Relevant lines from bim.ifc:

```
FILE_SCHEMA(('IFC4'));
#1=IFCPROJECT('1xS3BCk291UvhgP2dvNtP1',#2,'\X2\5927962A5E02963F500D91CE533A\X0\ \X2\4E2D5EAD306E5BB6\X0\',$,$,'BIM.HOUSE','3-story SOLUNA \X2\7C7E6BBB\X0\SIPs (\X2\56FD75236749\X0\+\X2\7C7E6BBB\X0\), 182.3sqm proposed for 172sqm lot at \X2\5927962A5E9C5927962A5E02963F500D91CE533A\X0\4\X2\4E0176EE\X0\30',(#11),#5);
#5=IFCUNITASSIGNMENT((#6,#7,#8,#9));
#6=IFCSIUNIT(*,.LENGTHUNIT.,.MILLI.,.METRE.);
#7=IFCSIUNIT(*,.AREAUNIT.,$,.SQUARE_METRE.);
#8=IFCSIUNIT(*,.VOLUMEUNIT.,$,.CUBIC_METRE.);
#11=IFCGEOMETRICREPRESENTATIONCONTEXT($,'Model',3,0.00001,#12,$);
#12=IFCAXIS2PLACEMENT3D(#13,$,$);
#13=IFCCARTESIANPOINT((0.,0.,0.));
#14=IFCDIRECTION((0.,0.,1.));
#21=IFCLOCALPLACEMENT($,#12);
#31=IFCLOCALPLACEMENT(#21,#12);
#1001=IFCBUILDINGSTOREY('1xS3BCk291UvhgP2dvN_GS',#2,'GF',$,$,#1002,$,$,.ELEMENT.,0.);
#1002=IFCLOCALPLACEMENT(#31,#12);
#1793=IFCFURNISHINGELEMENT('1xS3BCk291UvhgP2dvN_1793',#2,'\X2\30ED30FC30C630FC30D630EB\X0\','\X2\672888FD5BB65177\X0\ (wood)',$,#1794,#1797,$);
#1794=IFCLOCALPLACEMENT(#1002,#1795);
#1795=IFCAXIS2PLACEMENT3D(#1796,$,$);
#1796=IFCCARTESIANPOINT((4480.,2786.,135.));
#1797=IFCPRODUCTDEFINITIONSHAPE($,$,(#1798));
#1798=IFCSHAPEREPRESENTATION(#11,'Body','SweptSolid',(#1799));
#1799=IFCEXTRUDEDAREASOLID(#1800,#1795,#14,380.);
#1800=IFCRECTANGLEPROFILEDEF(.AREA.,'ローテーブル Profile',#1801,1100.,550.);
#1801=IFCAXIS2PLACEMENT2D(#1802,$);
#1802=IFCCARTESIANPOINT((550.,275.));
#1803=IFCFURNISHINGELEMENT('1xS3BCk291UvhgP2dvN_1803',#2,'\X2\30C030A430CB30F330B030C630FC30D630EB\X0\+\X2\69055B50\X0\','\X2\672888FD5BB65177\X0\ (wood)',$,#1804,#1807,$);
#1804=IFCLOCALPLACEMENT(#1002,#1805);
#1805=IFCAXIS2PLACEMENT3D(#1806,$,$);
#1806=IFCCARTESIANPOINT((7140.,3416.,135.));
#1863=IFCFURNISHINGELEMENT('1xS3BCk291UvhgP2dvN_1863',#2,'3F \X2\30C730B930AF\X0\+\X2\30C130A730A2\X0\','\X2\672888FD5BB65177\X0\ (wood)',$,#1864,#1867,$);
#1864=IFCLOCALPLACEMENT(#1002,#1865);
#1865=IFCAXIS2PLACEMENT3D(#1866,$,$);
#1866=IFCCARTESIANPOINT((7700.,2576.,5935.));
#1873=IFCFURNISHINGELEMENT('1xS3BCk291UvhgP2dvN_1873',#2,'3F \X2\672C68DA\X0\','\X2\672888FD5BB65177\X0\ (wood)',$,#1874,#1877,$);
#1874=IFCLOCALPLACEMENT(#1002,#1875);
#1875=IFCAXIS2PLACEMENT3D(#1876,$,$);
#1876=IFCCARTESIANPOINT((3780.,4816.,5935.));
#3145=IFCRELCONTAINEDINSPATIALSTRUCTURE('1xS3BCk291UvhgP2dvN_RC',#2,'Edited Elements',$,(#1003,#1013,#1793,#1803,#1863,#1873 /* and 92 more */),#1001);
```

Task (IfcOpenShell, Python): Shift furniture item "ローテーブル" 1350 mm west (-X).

```python
import ifcopenshell
import ifcopenshell.api.geometry
import ifcopenshell.util.placement
import ifcopenshell.util.unit

model = ifcopenshell.open("bim.ifc")
unit_scale = ifcopenshell.util.unit.calculate_unit_scale(model)

item = model.by_guid("1xS3BCk291UvhgP2dvN_1793")
matrix = ifcopenshell.util.placement.get_local_placement(item.ObjectPlacement)
matrix[0, 3] -= 1.35 / unit_scale
ifcopenshell.api.geometry.edit_object_placement(model, product=item, matrix=matrix, is_si=False)

print(ifcopenshell.util.placement.get_local_placement(item.ObjectPlacement).round(3) + 0.0)

model.write("bim-out.ifc")
```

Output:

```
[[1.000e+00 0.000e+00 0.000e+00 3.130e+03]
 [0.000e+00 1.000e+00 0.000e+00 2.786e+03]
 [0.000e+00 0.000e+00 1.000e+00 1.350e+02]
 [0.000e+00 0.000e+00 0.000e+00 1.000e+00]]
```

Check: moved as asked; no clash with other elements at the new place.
